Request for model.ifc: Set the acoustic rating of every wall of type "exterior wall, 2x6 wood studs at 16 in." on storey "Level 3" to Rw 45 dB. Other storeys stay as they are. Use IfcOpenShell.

First a look at what the model holds.

```python
import ifcopenshell
import ifcopenshell.util.element

model = ifcopenshell.open("model.ifc")
print(model.schema)
storey = next(s for s in model.by_type("IfcBuildingStorey") if s.Name == "Level 3")
walls = [e for e in ifcopenshell.util.element.get_decomposition(storey) if e.is_a("IfcWall")]
seen = {}
for e in walls:
    element_type = ifcopenshell.util.element.get_type(e)
    key = (element_type.Name if element_type != e and element_type else None, ifcopenshell.util.element.get_pset(e, "Pset_WallCommon", "AcousticRating"))
    seen[key] = seen.get(key, 0) + 1
for (name, value), count in sorted(seen.items(), key=str):
    print(count, "x", name, "|", value)
```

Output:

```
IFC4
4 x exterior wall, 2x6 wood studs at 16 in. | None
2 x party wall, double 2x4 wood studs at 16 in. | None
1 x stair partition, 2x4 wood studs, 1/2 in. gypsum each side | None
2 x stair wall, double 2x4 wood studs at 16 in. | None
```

```python
import ifcopenshell
import ifcopenshell.api.pset
import ifcopenshell.util.element

model = ifcopenshell.open("model.ifc")

storey = next(s for s in model.by_type("IfcBuildingStorey") if s.Name == "Level 3")
walls = [e for e in ifcopenshell.util.element.get_decomposition(storey) if e.is_a("IfcWall")]

count = 0
for e in walls:
    element_type = ifcopenshell.util.element.get_type(e)
    if element_type in (None, e) or element_type.Name != "exterior wall, 2x6 wood studs at 16 in.":
        continue
    # add_pset returns the element's existing set when there is one.
    pset = ifcopenshell.api.pset.add_pset(model, product=e, name="Pset_WallCommon")
    ifcopenshell.api.pset.edit_pset(model, pset=pset, properties={"AcousticRating": "Rw 45 dB"})
    count += 1

print(count, "walls updated")

model.write("model-out.ifc")
```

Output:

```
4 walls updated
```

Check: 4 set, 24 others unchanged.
